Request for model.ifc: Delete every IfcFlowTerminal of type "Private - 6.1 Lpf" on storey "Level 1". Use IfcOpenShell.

First a look at what the model holds.

```python
import ifcopenshell
import ifcopenshell.util.element

model = ifcopenshell.open("model.ifc")
print(model.schema)
storey = next(s for s in model.by_type("IfcBuildingStorey") if s.Name == "Level 1")
terminals = [e for e in ifcopenshell.util.element.get_decomposition(storey) if e.is_a("IfcFlowTerminal")]
seen = {}
for e in terminals:
    element_type = ifcopenshell.util.element.get_type(e)
    name = element_type.Name if element_type not in (None, e) else None
    seen[name] = seen.get(name, 0) + 1
for name, count in sorted(seen.items(), key=str):
    print(count, "x", name)
```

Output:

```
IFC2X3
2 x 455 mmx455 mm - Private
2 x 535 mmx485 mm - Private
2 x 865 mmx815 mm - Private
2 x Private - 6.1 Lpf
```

```python
import ifcopenshell
import ifcopenshell.api.root
import ifcopenshell.util.element

model = ifcopenshell.open("model.ifc")

storey = next(s for s in model.by_type("IfcBuildingStorey") if s.Name == "Level 1")
terminals = [e for e in ifcopenshell.util.element.get_decomposition(storey) if e.is_a("IfcFlowTerminal")]
targets = [e for e in terminals if (t := ifcopenshell.util.element.get_type(e)) not in (None, e) and t.Name == "Private - 6.1 Lpf"]

for e in targets:
    ifcopenshell.api.root.remove_product(model, product=e)
print(len(targets), "removed")

model.write("model_updated.ifc")
```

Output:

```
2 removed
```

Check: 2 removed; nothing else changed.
